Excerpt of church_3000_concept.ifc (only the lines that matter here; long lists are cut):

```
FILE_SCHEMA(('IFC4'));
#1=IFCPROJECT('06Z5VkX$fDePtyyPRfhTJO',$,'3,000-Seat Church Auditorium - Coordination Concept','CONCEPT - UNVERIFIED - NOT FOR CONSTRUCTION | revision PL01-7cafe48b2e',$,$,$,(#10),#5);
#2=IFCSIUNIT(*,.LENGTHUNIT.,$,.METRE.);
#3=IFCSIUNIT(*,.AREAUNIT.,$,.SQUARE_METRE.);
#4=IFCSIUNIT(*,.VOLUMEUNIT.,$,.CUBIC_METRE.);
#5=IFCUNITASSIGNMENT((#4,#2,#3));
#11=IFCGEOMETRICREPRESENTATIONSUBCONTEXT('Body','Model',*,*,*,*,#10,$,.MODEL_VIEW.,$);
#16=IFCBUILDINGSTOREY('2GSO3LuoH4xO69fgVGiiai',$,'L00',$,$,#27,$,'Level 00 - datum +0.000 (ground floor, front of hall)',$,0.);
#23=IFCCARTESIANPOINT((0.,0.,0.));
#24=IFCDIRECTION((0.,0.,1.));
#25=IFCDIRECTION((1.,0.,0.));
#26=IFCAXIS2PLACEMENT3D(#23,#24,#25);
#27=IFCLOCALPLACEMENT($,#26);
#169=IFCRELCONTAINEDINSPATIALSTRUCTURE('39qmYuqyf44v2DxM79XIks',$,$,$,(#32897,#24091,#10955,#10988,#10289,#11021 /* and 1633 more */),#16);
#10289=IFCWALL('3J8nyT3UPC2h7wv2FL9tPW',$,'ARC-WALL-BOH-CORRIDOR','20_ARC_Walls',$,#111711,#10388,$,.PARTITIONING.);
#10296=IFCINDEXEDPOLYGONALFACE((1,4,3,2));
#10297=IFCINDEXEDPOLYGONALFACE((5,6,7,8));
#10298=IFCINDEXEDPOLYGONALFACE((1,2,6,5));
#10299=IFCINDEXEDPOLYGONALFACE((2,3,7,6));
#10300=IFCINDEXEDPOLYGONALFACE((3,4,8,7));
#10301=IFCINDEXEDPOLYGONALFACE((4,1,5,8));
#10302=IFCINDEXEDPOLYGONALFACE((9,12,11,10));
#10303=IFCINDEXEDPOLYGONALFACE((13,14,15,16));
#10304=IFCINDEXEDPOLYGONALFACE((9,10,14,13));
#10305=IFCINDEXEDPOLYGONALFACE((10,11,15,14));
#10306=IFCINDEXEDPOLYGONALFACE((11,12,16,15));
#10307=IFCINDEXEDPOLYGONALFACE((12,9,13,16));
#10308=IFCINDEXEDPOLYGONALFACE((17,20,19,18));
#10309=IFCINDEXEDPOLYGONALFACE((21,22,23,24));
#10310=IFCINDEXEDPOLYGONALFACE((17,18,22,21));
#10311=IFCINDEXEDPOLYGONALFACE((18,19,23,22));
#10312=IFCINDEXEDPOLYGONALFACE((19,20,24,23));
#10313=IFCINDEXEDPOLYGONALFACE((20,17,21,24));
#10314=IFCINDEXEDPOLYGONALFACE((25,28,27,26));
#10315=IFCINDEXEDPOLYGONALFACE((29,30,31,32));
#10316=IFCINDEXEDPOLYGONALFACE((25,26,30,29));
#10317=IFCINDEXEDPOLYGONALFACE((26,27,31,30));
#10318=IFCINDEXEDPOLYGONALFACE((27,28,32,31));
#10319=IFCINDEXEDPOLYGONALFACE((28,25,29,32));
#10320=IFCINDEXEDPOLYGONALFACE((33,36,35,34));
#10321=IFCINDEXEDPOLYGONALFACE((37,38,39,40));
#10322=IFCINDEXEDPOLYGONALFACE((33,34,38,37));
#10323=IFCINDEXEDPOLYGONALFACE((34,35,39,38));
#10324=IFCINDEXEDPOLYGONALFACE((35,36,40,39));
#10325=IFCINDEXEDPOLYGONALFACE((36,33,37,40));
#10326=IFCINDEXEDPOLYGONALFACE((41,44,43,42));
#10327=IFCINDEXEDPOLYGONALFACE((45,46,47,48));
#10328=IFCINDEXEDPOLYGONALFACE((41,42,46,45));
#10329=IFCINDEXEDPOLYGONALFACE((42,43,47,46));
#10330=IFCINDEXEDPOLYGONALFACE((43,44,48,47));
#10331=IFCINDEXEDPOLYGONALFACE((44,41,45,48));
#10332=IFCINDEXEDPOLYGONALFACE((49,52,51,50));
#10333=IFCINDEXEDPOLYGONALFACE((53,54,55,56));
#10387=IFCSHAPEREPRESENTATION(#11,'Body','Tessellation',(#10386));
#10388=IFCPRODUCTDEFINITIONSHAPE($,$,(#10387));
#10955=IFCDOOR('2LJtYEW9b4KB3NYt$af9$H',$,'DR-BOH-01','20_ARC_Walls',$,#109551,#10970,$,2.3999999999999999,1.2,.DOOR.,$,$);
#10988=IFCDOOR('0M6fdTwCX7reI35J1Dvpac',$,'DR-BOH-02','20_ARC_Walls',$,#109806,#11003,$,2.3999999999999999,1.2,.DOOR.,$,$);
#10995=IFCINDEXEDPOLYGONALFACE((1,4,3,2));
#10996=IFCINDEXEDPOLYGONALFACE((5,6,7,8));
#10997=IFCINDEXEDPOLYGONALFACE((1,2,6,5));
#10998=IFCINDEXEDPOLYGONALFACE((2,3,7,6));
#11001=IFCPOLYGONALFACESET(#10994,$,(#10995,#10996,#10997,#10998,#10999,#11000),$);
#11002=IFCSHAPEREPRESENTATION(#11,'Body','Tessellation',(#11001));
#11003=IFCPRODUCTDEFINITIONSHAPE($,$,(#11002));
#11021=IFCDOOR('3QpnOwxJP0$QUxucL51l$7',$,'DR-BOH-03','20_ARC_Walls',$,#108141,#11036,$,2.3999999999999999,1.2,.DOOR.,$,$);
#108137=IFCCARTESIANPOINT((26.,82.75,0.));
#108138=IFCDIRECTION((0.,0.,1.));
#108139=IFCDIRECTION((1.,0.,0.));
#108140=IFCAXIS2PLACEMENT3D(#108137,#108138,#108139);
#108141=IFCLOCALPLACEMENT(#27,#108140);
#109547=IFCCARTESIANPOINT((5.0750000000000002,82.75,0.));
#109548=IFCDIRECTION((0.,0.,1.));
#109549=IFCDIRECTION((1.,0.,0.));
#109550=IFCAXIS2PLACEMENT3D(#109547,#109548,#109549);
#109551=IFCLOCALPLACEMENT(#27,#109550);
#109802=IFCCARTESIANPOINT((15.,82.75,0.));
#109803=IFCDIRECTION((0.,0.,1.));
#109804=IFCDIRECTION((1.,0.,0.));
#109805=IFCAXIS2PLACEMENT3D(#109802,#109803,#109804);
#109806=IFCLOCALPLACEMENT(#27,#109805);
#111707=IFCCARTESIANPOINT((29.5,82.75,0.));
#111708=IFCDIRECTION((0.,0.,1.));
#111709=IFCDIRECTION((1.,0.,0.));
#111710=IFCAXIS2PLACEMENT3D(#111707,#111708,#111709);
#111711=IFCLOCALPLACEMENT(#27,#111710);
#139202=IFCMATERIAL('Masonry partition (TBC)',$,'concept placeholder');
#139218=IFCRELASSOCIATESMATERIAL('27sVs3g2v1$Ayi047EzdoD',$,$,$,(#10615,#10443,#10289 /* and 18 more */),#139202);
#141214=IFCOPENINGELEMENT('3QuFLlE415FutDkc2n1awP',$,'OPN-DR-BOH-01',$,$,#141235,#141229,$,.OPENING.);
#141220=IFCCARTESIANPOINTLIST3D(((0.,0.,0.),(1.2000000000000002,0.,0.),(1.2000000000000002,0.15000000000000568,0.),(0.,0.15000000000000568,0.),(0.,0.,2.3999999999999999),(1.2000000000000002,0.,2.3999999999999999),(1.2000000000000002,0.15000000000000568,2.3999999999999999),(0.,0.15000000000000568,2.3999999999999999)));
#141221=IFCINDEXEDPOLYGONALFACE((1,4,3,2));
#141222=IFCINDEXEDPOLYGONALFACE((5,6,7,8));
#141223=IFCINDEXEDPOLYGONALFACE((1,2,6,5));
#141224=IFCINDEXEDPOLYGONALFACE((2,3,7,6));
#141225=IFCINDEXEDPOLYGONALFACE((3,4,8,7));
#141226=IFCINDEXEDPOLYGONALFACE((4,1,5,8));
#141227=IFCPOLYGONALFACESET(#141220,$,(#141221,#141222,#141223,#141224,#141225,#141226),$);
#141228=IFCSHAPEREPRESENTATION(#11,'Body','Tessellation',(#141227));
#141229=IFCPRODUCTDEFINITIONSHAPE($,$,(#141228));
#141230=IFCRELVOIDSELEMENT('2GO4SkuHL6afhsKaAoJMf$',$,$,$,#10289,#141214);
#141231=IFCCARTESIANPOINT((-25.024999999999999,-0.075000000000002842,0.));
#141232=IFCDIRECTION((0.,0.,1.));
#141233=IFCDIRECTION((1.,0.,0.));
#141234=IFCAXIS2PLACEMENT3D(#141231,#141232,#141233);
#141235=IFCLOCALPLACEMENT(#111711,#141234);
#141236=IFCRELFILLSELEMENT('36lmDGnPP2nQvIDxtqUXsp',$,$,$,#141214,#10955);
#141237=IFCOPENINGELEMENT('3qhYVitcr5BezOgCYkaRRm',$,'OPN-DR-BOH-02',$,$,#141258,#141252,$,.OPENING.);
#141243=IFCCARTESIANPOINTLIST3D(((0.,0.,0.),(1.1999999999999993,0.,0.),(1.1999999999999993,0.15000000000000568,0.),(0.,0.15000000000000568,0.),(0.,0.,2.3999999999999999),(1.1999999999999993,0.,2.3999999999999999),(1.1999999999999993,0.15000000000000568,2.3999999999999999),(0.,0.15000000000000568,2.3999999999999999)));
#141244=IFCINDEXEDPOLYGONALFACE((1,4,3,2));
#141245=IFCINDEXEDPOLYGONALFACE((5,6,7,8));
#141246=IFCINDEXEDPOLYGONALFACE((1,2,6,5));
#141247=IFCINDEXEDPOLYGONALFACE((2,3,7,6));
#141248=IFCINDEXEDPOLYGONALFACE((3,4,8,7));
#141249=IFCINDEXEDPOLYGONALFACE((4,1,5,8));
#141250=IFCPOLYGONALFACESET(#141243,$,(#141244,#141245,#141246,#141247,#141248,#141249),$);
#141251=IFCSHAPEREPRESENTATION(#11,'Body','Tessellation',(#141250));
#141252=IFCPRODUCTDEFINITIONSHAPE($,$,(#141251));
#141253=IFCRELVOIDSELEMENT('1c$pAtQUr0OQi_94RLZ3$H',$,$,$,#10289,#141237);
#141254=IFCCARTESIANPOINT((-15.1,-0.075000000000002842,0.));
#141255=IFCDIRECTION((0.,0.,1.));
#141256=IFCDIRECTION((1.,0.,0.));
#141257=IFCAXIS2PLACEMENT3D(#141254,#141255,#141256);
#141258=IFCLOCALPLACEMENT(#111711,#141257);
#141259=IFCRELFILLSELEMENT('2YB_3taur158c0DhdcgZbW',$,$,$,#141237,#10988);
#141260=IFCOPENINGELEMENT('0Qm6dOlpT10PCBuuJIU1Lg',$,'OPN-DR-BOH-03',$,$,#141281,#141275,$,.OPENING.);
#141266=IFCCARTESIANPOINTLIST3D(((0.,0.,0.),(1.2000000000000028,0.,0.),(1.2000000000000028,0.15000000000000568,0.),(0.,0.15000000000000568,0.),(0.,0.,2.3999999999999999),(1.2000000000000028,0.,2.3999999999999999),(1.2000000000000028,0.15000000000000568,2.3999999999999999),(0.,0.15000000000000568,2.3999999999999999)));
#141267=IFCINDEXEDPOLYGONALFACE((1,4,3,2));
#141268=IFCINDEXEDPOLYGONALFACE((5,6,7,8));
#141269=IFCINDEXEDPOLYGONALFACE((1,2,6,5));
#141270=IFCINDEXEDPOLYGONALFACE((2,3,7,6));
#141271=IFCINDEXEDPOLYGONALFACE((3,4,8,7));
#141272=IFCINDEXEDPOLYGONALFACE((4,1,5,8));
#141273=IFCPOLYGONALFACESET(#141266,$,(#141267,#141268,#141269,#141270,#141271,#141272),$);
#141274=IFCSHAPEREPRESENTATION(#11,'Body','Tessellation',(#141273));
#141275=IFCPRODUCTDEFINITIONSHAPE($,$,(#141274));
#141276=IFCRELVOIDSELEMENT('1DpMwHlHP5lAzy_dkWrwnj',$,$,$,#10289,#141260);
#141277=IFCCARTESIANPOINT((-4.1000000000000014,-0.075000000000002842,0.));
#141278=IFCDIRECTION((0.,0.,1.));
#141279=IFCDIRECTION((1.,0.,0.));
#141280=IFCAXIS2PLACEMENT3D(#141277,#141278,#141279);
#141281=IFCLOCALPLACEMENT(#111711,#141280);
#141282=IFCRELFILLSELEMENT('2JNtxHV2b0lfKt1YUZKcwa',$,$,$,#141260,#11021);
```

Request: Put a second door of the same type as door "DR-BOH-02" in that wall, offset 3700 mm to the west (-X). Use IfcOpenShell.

```python
import ifcopenshell
import ifcopenshell.api.feature
import ifcopenshell.api.geometry
import ifcopenshell.api.root
import ifcopenshell.geom
import ifcopenshell.util.element
import ifcopenshell.util.placement
import ifcopenshell.util.shape
import ifcopenshell.util.unit

model = ifcopenshell.open("church_3000_concept.ifc")
unit_scale = ifcopenshell.util.unit.calculate_unit_scale(model)
settings = ifcopenshell.geom.settings()


def volume(element):
    """Net volume in cubic metres, openings subtracted."""
    shape = ifcopenshell.geom.create_shape(settings, element)
    return ifcopenshell.util.shape.get_volume(shape.geometry)


door = model.by_id(10988)
opening = door.FillsVoids[0].RelatingOpeningElement
wall = opening.VoidsElements[0].RelatingBuildingElement
before = volume(wall)
shift = ifcopenshell.util.placement.get_local_placement(wall.ObjectPlacement)[:3, 0] * -3.7 / unit_scale

# copy_class copies the void relationship, type, container and properties, but no geometry.
new_opening = ifcopenshell.api.root.copy_class(model, product=opening)
new_opening.Representation = ifcopenshell.util.element.copy_deep(
    model, opening.Representation, exclude=["IfcGeometricRepresentationContext", "IfcRepresentationMap"]
)
new_door = ifcopenshell.api.root.copy_class(model, product=door)
new_door.Representation = ifcopenshell.util.element.copy_deep(
    model, door.Representation, exclude=["IfcGeometricRepresentationContext", "IfcRepresentationMap"]
)
ifcopenshell.api.feature.add_filling(model, opening=new_opening, element=new_door)

for old, new in ((opening, new_opening), (door, new_door)):
    matrix = ifcopenshell.util.placement.get_local_placement(old.ObjectPlacement)
    matrix[:3, 3] += shift
    ifcopenshell.api.geometry.edit_object_placement(model, product=new, matrix=matrix, is_si=False)

after = volume(wall)

print(f"wall volume {before:.3f} -> {after:.3f} m3")

model.write("church_3000_concept_rev.ifc")
```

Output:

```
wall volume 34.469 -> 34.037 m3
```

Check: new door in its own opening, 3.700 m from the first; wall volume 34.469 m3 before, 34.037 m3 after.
